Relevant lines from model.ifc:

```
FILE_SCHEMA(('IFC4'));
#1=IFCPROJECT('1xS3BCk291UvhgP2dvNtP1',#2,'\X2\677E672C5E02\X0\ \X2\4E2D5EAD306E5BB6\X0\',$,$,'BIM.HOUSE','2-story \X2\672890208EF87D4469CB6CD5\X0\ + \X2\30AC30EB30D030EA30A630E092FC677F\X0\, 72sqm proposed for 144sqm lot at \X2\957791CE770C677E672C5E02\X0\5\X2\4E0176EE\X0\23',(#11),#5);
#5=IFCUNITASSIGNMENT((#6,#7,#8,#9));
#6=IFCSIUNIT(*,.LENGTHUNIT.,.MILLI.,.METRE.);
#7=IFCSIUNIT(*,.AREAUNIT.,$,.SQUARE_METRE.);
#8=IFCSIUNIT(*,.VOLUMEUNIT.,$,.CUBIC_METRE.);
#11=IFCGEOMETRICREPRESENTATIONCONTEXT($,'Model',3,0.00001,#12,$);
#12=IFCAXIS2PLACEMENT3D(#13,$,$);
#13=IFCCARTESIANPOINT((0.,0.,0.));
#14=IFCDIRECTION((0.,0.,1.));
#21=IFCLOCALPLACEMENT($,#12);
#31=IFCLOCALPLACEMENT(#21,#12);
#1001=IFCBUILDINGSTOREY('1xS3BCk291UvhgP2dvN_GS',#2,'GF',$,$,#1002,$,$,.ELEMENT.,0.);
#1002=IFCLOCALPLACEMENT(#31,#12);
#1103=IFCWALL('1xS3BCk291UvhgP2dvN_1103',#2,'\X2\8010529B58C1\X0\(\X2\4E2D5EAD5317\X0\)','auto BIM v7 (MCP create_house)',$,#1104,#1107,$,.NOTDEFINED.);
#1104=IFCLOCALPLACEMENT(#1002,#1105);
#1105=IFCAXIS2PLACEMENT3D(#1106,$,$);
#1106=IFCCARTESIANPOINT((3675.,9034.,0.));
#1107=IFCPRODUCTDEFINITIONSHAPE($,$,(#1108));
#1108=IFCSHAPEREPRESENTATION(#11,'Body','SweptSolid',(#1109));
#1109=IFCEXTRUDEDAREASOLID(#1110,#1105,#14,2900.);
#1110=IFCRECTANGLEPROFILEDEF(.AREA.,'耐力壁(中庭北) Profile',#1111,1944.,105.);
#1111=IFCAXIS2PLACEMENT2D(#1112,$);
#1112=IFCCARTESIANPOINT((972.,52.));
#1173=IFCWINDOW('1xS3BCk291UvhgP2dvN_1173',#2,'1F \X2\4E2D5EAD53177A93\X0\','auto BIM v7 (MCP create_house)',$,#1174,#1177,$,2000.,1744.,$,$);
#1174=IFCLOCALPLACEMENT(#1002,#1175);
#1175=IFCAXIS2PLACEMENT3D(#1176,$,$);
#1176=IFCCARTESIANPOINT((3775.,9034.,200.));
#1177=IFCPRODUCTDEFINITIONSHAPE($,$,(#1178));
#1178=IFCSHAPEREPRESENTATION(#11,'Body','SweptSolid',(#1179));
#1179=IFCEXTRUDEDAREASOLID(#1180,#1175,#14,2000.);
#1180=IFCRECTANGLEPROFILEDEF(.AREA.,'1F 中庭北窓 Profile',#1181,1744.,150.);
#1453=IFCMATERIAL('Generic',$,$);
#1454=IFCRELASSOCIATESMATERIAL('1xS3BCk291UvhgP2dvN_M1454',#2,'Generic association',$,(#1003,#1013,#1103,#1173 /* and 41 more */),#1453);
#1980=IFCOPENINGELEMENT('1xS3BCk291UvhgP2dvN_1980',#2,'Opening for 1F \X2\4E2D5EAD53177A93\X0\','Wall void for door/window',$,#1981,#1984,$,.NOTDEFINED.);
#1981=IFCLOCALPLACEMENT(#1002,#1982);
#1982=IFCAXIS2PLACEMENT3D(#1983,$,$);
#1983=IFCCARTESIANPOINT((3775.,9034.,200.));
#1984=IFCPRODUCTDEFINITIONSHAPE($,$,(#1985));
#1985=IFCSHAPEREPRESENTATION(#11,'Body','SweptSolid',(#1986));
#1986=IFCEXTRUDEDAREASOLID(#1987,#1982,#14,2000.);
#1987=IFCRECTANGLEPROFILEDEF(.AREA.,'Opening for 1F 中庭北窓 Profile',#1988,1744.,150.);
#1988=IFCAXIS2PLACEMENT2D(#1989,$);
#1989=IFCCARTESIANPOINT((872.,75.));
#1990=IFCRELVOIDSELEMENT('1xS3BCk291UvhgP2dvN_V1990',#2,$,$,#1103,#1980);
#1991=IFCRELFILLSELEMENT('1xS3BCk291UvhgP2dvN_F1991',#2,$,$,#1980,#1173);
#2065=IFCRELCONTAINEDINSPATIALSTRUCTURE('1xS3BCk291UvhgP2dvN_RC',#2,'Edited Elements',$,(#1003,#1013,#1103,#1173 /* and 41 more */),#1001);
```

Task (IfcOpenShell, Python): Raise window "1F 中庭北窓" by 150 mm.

```python
import numpy as np
import ifcopenshell
import ifcopenshell.api.geometry
import ifcopenshell.util.placement
import ifcopenshell.util.unit

model = ifcopenshell.open("model.ifc")
unit_scale = ifcopenshell.util.unit.calculate_unit_scale(model)

window = model.by_guid("1xS3BCk291UvhgP2dvN_1173")
opening = window.FillsVoids[0].RelatingOpeningElement
dz = 150.0

shift = np.array([0.0, 0.0, dz])
# The window is not placed relative to its opening, so move both.
for product in (opening, window):
    matrix = ifcopenshell.util.placement.get_local_placement(product.ObjectPlacement)
    matrix[:3, 3] += shift
    ifcopenshell.api.geometry.edit_object_placement(model, product=product, matrix=matrix, is_si=False)

print(f"moved by {dz * unit_scale:+.3f} m")

model.write("model_edited.ifc")
```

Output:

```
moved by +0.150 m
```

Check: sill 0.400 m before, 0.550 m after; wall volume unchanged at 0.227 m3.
